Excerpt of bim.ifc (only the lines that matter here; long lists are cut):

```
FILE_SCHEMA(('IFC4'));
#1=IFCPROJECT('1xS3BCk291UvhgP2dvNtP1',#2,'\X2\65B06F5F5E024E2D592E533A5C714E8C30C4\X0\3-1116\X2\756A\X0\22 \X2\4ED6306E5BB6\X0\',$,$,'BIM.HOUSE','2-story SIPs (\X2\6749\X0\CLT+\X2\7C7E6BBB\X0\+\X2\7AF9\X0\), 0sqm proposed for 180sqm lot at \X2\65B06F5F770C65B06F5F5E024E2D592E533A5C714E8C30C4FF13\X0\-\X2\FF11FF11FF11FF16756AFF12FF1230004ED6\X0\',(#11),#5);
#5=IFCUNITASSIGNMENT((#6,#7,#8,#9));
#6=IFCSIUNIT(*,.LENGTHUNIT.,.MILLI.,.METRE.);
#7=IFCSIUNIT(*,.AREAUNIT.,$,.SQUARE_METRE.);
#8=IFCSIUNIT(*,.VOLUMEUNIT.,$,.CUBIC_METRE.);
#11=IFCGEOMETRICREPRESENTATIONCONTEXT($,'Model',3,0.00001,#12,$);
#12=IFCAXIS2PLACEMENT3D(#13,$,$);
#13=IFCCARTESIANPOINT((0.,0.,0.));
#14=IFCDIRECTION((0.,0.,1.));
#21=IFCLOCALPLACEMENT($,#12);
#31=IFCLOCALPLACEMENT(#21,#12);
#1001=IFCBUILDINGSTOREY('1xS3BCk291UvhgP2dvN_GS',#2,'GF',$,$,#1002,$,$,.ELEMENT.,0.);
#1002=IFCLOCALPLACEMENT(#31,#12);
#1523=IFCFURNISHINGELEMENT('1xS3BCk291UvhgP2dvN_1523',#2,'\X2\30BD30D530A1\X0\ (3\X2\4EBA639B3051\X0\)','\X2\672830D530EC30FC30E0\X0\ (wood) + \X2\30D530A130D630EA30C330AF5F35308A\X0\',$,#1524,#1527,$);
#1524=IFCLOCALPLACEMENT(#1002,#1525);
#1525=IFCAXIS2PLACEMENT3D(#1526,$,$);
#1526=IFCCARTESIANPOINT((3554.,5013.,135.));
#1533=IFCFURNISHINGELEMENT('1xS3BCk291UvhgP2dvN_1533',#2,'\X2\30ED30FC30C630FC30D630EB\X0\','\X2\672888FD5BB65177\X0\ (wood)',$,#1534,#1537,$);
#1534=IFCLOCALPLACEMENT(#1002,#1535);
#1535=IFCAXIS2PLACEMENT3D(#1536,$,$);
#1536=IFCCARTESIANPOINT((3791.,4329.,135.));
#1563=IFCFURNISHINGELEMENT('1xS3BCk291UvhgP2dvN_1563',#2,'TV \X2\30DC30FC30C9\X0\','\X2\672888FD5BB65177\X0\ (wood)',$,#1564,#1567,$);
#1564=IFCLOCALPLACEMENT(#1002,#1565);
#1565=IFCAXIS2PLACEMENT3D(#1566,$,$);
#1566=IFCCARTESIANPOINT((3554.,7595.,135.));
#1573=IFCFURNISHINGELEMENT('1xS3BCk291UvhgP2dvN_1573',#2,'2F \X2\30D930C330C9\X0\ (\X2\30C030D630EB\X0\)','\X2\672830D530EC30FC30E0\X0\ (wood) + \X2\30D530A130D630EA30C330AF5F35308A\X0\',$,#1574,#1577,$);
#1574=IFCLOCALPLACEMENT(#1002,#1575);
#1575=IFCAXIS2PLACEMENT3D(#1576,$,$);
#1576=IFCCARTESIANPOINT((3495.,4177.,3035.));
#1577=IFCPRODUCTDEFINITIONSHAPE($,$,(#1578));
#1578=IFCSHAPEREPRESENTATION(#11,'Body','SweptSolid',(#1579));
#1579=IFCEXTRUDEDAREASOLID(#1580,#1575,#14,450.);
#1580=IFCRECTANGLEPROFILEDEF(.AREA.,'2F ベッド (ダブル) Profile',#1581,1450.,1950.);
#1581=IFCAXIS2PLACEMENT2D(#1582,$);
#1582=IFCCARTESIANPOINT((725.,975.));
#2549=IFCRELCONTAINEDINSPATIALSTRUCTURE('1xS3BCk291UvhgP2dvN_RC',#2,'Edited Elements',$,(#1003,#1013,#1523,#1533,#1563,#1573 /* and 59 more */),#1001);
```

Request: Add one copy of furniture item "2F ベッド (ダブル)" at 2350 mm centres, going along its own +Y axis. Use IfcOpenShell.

```python
import ifcopenshell
import ifcopenshell.api.geometry
import ifcopenshell.api.root
import ifcopenshell.util.element
import ifcopenshell.util.placement
import ifcopenshell.util.unit

model = ifcopenshell.open("bim.ifc")
unit_scale = ifcopenshell.util.unit.calculate_unit_scale(model)


def reuse_history(source, copy):
    """copy_class also copies each property set's owner history, people and application; keep the originals."""
    for rel in copy.IsDefinedBy:
        if rel.is_a("IfcRelDefinesByProperties") and (history := rel.RelatingPropertyDefinition.OwnerHistory):
            rel.RelatingPropertyDefinition.OwnerHistory = source.OwnerHistory
            ifcopenshell.util.element.remove_deep2(model, history)


source = model.by_guid("1xS3BCk291UvhgP2dvN_1573")
base = ifcopenshell.util.placement.get_local_placement(source.ObjectPlacement)
step = base[:3, 1] * 2.35 / unit_scale

for i in range(1, 2):
    copy = ifcopenshell.api.root.copy_class(model, product=source)
    copy.Representation = ifcopenshell.util.element.copy_deep(
        model, source.Representation, exclude=["IfcGeometricRepresentationContext", "IfcRepresentationMap"]
    )
    reuse_history(source, copy)
    matrix = base.copy()
    matrix[:3, 3] += i * step
    print("added at", matrix[:3, 3].round(3) + 0.0)
    ifcopenshell.api.geometry.edit_object_placement(model, product=copy, matrix=matrix, is_si=False)

model.write("bim-out.ifc")
```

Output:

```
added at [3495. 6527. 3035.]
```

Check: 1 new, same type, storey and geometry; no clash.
